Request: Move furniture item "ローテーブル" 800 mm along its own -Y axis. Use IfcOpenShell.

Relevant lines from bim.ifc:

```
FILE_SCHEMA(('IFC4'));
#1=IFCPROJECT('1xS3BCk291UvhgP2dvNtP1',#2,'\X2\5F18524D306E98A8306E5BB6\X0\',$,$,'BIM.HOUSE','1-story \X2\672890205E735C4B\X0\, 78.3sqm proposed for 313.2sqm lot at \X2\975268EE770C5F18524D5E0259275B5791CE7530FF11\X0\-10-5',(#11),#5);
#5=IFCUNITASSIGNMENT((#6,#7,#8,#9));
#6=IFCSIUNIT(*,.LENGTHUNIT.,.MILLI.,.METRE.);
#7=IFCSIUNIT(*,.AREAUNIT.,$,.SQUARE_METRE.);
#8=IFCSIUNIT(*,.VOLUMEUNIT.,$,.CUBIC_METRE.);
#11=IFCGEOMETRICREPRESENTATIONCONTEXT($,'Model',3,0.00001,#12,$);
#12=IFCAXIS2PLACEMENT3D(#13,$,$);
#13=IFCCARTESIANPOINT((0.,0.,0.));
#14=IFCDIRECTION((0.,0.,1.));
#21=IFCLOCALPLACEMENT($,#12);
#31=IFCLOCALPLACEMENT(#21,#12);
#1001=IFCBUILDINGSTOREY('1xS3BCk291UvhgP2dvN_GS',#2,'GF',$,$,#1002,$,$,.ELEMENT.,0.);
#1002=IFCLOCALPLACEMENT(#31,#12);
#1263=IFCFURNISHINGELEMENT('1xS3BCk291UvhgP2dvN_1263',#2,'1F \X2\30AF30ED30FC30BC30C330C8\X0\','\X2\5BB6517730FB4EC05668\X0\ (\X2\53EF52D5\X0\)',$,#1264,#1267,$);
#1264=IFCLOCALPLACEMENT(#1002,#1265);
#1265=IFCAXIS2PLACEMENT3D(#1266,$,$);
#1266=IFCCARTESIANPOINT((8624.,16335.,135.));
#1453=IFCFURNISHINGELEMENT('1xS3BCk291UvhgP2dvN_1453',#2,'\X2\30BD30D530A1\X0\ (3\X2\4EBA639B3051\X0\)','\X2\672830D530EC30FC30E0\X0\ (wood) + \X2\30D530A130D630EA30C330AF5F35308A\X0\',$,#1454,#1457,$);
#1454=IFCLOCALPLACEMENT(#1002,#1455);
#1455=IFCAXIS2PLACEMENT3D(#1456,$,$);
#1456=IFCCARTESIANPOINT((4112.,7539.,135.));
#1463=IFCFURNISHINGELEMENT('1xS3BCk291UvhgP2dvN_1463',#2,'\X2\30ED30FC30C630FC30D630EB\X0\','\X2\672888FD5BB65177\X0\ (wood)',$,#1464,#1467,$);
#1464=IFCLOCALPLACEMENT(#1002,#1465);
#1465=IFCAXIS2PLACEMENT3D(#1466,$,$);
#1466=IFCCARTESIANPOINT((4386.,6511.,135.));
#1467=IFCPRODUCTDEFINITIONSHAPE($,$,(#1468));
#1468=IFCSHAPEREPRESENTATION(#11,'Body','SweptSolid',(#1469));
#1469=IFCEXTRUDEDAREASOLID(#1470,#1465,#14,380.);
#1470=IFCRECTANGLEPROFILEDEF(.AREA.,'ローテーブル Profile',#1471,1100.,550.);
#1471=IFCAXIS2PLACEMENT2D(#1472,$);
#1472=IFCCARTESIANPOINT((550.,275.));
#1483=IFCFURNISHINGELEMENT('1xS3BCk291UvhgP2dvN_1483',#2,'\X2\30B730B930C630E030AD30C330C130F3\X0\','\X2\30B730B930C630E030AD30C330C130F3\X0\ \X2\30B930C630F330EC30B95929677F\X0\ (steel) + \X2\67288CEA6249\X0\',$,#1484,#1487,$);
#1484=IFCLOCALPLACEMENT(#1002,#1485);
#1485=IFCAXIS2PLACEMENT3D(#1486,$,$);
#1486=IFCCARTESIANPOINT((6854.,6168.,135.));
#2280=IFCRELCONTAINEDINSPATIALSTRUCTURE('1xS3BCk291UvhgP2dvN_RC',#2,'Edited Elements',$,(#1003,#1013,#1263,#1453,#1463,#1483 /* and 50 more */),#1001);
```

```python
import ifcopenshell
import ifcopenshell.api.geometry
import ifcopenshell.util.placement
import ifcopenshell.util.unit

model = ifcopenshell.open("bim.ifc")
unit_scale = ifcopenshell.util.unit.calculate_unit_scale(model)

item = model.by_guid("1xS3BCk291UvhgP2dvN_1463")
matrix = ifcopenshell.util.placement.get_local_placement(item.ObjectPlacement)
matrix[:3, 3] -= matrix[:3, 1] * 0.8 / unit_scale
ifcopenshell.api.geometry.edit_object_placement(model, product=item, matrix=matrix, is_si=False)

print(ifcopenshell.util.placement.get_local_placement(item.ObjectPlacement).round(3) + 0.0)

model.write("bim_rev.ifc")
```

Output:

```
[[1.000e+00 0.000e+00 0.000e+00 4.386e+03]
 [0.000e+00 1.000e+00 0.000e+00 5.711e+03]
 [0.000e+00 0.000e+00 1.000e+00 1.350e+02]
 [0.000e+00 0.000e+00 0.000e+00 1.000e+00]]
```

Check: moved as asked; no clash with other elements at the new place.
